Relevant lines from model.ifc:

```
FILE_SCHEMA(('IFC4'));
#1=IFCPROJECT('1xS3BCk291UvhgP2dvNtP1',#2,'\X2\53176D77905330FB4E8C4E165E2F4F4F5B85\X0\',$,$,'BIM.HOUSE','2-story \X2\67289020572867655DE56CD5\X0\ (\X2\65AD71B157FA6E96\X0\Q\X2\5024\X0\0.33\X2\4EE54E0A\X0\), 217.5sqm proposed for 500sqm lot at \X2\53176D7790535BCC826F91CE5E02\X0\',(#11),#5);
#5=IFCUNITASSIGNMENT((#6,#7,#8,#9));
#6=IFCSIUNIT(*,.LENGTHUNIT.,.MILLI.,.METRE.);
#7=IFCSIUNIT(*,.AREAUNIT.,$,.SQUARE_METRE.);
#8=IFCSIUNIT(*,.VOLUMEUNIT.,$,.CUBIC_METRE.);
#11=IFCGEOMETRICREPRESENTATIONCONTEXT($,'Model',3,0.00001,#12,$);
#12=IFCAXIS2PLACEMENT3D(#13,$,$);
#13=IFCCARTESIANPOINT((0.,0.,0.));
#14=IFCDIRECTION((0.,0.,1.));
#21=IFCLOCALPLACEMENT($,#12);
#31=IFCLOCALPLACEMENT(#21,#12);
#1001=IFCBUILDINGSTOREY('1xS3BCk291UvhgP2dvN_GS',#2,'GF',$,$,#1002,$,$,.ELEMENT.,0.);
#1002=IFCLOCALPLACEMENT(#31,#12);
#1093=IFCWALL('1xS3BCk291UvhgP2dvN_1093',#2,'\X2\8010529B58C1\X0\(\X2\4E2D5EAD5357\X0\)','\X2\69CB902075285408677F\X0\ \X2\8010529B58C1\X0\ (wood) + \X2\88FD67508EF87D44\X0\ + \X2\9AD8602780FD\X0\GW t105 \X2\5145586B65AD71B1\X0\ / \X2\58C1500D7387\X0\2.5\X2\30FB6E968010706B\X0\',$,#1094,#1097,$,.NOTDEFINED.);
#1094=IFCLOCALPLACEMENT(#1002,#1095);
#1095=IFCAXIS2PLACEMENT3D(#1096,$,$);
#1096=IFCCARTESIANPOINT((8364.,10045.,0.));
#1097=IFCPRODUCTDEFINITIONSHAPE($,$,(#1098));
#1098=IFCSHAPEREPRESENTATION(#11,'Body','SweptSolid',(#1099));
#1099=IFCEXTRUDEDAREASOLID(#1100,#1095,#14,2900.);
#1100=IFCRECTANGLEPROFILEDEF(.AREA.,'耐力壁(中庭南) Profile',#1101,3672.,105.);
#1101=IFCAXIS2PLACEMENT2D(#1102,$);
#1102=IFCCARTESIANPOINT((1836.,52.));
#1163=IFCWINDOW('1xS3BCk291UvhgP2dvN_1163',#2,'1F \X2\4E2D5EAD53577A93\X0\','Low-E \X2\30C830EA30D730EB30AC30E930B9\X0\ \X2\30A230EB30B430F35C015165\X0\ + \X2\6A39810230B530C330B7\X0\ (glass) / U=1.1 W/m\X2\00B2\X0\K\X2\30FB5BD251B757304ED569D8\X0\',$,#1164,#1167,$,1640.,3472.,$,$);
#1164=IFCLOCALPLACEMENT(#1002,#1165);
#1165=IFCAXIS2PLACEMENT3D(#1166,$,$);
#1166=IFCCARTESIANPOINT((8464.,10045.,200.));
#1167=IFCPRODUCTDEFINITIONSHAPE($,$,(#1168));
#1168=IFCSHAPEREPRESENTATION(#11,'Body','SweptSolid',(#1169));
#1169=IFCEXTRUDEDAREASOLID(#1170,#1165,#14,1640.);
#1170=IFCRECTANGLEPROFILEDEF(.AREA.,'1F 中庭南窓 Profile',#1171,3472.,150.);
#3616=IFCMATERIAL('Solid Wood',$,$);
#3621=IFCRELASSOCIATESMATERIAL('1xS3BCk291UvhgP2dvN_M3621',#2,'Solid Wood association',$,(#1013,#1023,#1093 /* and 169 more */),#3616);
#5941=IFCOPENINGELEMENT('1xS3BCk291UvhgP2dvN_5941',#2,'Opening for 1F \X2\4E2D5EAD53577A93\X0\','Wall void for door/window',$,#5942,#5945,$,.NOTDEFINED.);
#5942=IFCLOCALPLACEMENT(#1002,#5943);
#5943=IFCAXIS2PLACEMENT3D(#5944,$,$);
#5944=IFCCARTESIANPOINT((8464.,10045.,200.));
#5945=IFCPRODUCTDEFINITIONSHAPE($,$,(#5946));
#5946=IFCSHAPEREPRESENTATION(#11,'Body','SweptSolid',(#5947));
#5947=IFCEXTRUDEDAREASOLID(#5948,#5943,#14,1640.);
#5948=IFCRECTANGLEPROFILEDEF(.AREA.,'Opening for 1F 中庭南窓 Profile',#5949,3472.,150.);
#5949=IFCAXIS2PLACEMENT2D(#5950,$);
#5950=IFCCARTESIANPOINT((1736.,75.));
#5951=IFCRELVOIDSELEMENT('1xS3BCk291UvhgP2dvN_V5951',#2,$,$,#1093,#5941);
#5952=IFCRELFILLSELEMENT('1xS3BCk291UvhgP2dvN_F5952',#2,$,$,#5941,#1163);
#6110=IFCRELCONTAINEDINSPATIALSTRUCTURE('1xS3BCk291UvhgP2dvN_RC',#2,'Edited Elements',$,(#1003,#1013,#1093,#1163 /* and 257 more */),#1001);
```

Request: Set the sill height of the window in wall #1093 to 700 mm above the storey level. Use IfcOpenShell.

```python
import numpy as np
import ifcopenshell
import ifcopenshell.api.geometry
import ifcopenshell.geom
import ifcopenshell.util.element
import ifcopenshell.util.placement
import ifcopenshell.util.shape
import ifcopenshell.util.unit

model = ifcopenshell.open("model.ifc")
unit_scale = ifcopenshell.util.unit.calculate_unit_scale(model)

window = model.by_id(1163)
opening = window.FillsVoids[0].RelatingOpeningElement
storey = ifcopenshell.util.element.get_container(window, ifc_class="IfcBuildingStorey")
level = ifcopenshell.util.placement.get_local_placement(storey.ObjectPlacement)[2, 3]

# The opening's origin need not be at the sill, so measure its lowest point.
shape = ifcopenshell.geom.create_shape(ifcopenshell.geom.settings(), opening)
bottom = ifcopenshell.util.shape.get_shape_bottom_elevation(shape, shape.geometry) / unit_scale
dz = level + 700.0 - bottom

shift = np.array([0.0, 0.0, dz])
# The window is not placed relative to its opening, so move both.
for product in (opening, window):
    matrix = ifcopenshell.util.placement.get_local_placement(product.ObjectPlacement)
    matrix[:3, 3] += shift
    ifcopenshell.api.geometry.edit_object_placement(model, product=product, matrix=matrix, is_si=False)

print(f"moved by {dz * unit_scale:+.3f} m")

model.write("model_edited.ifc")
```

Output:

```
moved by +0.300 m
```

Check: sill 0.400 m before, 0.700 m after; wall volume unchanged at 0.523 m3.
